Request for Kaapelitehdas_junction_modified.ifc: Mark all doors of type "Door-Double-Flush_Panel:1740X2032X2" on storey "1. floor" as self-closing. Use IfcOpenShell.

First a look at what the model holds.

```python
import ifcopenshell
import ifcopenshell.util.element

model = ifcopenshell.open("Kaapelitehdas_junction_modified.ifc")
print(model.schema)
storey = next(s for s in model.by_type("IfcBuildingStorey") if s.Name == "1. floor")
doors = [e for e in ifcopenshell.util.element.get_decomposition(storey) if e.is_a("IfcDoor")]
seen = {}
for e in doors:
    element_type = ifcopenshell.util.element.get_type(e)
    key = (element_type.Name if element_type != e and element_type else None, ifcopenshell.util.element.get_pset(e, "Pset_DoorCommon", "SelfClosing"))
    seen[key] = seen.get(key, 0) + 1
for (name, value), count in sorted(seen.items(), key=str):
    print(count, "x", name, "|", value)
```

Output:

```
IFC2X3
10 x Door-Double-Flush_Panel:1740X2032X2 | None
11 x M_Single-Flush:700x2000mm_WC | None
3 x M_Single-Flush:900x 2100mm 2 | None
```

```python
import ifcopenshell
import ifcopenshell.api.pset
import ifcopenshell.util.element

model = ifcopenshell.open("Kaapelitehdas_junction_modified.ifc")

storey = next(s for s in model.by_type("IfcBuildingStorey") if s.Name == "1. floor")
doors = [e for e in ifcopenshell.util.element.get_decomposition(storey) if e.is_a("IfcDoor")]

count = 0
for e in doors:
    element_type = ifcopenshell.util.element.get_type(e)
    if element_type in (None, e) or element_type.Name != "Door-Double-Flush_Panel:1740X2032X2":
        continue
    # add_pset returns the element's existing set when there is one.
    pset = ifcopenshell.api.pset.add_pset(model, product=e, name="Pset_DoorCommon")
    ifcopenshell.api.pset.edit_pset(model, pset=pset, properties={"SelfClosing": True})
    count += 1

print(count, "doors updated")

model.write("Kaapelitehdas_junction_modified-out.ifc")
```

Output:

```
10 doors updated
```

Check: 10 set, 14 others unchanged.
